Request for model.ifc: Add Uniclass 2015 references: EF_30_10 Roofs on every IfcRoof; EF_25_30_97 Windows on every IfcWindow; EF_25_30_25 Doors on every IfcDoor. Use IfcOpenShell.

First a look at what the model holds.

```python
import ifcopenshell

model = ifcopenshell.open("model.ifc")
print(model.schema)
print("classifications:", [c.Name for c in model.by_type("IfcClassification")])
for ifc_class in ("IfcDoor", "IfcRoof", "IfcStair", "IfcWall", "IfcWindow"):
    print(ifc_class, len(model.by_type(ifc_class)))
```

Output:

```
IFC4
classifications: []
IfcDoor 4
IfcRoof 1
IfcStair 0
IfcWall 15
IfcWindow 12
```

```python
import ifcopenshell
import ifcopenshell.api.classification

model = ifcopenshell.open("model.ifc")

system = ifcopenshell.api.classification.add_classification(model, classification="Uniclass 2015")

codes = {
    "IfcRoof": ("EF_30_10", "Roofs"),
    "IfcWindow": ("EF_25_30_97", "Windows"),
    "IfcDoor": ("EF_25_30_25", "Doors"),
}
for ifc_class, (code, name) in codes.items():
    products = model.by_type(ifc_class)
    ifcopenshell.api.classification.add_reference(
        model, products=products, classification=system, identification=code, name=name
    )
    print(code, len(products))

model.write("model_rev.ifc")
```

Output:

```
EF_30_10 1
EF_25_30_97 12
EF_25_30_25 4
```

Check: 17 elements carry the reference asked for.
